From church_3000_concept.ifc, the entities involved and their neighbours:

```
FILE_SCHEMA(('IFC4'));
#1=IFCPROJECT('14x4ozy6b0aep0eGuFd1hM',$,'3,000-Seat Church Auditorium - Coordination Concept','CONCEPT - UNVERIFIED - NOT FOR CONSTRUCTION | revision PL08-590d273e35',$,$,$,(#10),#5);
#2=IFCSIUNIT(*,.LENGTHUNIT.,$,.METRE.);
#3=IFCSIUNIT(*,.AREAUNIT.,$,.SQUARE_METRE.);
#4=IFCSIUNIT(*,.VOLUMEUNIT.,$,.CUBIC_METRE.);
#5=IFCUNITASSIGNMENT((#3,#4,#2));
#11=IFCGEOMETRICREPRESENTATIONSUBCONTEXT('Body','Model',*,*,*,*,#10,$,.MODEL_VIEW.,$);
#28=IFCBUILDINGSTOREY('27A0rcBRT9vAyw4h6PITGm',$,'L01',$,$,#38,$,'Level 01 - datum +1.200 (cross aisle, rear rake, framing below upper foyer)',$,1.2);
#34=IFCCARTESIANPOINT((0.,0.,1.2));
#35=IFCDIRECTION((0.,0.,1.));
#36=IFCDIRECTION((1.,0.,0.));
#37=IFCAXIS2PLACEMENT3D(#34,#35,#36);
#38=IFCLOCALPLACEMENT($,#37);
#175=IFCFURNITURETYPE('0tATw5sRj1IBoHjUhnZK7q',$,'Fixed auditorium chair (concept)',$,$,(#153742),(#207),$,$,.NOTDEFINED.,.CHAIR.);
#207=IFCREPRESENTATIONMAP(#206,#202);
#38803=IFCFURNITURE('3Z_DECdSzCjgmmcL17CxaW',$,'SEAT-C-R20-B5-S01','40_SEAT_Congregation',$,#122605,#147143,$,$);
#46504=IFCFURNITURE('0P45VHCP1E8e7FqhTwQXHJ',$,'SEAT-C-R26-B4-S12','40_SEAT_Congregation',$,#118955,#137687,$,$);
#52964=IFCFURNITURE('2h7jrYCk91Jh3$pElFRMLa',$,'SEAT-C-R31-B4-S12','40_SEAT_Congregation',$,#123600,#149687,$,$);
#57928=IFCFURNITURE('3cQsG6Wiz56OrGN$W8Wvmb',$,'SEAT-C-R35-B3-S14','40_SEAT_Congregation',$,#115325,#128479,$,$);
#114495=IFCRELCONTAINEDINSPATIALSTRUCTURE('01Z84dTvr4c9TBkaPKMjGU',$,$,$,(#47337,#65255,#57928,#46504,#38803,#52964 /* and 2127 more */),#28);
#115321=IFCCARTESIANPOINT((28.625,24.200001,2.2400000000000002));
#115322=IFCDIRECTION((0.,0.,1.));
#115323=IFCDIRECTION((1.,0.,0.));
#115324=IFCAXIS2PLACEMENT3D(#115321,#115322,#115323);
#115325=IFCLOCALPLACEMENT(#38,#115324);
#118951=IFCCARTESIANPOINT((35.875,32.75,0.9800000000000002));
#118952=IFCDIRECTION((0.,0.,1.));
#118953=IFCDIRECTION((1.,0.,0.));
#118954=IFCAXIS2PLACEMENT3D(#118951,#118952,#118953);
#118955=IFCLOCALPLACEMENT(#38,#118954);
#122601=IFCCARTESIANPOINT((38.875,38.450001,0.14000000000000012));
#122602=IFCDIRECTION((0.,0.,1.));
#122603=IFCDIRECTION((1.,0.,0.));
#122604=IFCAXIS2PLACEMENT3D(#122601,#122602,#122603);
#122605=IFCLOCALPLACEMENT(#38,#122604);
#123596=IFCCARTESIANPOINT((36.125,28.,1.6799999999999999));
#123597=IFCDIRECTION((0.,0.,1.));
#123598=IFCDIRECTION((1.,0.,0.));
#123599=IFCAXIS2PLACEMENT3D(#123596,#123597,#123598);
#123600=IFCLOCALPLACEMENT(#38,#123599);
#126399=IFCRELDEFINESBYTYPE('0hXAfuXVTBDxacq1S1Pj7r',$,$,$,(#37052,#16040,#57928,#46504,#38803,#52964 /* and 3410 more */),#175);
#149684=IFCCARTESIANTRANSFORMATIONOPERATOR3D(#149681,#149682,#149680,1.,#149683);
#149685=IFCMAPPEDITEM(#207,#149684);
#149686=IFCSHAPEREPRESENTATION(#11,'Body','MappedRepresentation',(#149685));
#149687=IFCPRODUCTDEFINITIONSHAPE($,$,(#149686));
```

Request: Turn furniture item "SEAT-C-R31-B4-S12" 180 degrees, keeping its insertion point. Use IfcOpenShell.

```python
import ifcopenshell
import ifcopenshell.api.geometry
import ifcopenshell.util.placement

model = ifcopenshell.open("church_3000_concept.ifc")

item = model.by_guid("2h7jrYCk91Jh3$pElFRMLa")
matrix = ifcopenshell.util.placement.get_local_placement(item.ObjectPlacement)
matrix = matrix @ ifcopenshell.util.placement.rotation(180, "Z")
ifcopenshell.api.geometry.edit_object_placement(model, product=item, matrix=matrix, is_si=False)

print(ifcopenshell.util.placement.get_local_placement(item.ObjectPlacement).round(3) + 0.0)

model.write("church_3000_concept-out.ifc")
```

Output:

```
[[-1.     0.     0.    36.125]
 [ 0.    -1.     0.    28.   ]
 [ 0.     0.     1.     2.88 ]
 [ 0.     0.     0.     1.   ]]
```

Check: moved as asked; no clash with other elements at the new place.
